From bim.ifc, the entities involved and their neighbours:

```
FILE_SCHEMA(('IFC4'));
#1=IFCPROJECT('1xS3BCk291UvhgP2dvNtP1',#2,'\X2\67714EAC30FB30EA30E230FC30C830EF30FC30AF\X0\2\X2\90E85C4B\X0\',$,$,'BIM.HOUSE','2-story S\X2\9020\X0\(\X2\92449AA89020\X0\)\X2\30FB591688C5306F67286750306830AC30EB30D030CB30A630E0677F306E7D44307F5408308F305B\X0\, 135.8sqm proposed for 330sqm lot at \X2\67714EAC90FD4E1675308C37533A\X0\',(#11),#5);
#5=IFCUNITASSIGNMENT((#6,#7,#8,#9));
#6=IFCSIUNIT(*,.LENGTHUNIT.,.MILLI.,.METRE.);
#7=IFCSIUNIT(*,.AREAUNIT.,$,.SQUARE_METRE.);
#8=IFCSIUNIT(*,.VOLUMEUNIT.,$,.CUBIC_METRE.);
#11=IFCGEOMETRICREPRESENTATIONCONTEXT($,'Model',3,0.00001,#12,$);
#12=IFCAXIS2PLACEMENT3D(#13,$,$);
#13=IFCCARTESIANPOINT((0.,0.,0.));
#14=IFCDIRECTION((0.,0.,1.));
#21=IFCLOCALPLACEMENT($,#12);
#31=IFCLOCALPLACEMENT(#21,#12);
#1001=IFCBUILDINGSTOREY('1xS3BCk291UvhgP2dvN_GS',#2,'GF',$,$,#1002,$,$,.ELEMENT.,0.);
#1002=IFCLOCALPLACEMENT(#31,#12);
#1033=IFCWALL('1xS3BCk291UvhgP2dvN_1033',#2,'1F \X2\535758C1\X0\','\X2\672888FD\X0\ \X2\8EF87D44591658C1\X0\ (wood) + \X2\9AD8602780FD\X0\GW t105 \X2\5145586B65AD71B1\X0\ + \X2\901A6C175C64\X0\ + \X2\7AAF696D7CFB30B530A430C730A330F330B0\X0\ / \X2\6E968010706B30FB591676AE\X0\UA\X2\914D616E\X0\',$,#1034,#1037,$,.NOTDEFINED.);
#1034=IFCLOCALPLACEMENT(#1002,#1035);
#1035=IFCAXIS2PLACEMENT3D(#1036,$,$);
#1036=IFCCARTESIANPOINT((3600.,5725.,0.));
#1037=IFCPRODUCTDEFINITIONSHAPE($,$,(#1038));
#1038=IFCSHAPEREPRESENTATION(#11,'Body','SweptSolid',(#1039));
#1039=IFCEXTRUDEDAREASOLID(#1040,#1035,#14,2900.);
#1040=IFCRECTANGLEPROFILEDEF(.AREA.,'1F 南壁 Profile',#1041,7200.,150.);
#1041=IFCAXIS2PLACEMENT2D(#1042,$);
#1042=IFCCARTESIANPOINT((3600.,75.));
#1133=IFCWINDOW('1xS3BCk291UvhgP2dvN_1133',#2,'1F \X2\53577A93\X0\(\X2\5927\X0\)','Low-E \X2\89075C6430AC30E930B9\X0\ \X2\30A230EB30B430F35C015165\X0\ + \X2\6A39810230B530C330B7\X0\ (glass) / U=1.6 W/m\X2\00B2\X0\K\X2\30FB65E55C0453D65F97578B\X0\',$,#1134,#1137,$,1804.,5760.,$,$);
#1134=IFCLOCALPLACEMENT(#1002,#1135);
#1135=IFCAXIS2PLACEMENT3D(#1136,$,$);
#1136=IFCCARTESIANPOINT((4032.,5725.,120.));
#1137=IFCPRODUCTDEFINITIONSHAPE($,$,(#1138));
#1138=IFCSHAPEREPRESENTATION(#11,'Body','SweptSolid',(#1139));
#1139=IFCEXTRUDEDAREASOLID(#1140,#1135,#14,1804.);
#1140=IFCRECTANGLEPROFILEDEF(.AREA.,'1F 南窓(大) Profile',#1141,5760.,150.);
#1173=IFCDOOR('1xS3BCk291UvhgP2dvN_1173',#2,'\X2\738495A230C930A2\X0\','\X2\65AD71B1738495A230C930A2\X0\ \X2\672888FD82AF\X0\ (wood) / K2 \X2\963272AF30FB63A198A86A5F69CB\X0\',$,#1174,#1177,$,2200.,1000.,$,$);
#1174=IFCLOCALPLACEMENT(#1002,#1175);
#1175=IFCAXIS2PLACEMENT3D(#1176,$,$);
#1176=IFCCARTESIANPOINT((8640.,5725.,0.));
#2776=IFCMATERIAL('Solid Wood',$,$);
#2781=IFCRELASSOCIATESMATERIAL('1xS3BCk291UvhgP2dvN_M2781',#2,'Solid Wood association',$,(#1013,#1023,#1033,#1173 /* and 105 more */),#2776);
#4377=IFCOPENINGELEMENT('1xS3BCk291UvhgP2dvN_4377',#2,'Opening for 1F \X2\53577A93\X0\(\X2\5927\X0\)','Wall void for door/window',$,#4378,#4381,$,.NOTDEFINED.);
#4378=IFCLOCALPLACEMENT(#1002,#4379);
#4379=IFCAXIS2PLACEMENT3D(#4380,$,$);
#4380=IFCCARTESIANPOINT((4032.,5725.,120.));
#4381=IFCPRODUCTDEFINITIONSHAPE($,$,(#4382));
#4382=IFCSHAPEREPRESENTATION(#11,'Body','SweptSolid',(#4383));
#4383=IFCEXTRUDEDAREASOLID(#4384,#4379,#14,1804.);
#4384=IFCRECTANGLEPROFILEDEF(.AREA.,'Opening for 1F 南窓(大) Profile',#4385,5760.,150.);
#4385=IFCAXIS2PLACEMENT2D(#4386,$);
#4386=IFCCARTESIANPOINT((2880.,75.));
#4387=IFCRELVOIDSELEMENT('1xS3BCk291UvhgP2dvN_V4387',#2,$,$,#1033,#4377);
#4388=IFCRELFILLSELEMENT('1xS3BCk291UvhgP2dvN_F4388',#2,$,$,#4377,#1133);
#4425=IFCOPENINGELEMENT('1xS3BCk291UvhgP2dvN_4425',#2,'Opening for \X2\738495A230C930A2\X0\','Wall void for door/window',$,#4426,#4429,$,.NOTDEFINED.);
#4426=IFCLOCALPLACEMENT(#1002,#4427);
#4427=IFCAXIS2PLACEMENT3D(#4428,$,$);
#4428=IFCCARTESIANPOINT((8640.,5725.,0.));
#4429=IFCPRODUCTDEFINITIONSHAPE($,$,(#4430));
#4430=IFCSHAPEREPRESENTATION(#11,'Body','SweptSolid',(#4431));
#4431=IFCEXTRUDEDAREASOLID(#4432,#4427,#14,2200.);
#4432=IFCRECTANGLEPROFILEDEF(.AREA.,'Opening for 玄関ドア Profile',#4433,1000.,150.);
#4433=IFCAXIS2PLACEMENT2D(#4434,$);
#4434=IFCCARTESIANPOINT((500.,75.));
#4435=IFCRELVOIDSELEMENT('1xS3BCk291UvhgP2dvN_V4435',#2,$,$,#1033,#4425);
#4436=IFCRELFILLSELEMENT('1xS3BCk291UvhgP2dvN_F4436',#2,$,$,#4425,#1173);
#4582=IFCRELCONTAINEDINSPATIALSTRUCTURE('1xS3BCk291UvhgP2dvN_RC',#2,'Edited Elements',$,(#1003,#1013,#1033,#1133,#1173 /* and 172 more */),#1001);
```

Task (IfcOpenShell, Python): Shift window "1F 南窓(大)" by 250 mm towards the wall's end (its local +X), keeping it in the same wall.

```python
import ifcopenshell
import ifcopenshell.api.geometry
import ifcopenshell.util.placement
import ifcopenshell.util.unit

model = ifcopenshell.open("bim.ifc")
unit_scale = ifcopenshell.util.unit.calculate_unit_scale(model)

window = model.by_guid("1xS3BCk291UvhgP2dvN_1133")
opening = window.FillsVoids[0].RelatingOpeningElement
wall = opening.VoidsElements[0].RelatingBuildingElement

wall_matrix = ifcopenshell.util.placement.get_local_placement(wall.ObjectPlacement)
shift = wall_matrix[:3, 0] * 0.25 / unit_scale
before = ifcopenshell.util.placement.get_local_placement(window.ObjectPlacement)[:3, 3].copy()

# The window is not placed relative to its opening, so move both.
for product in (opening, window):
    matrix = ifcopenshell.util.placement.get_local_placement(product.ObjectPlacement)
    matrix[:3, 3] += shift
    ifcopenshell.api.geometry.edit_object_placement(model, product=product, matrix=matrix, is_si=False)

after = ifcopenshell.util.placement.get_local_placement(window.ObjectPlacement)[:3, 3]
print("window moved by", (after - before).round(3) + 0.0)

model.write("bim_v2.ifc")
```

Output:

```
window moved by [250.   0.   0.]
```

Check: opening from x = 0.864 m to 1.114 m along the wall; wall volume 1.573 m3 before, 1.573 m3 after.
